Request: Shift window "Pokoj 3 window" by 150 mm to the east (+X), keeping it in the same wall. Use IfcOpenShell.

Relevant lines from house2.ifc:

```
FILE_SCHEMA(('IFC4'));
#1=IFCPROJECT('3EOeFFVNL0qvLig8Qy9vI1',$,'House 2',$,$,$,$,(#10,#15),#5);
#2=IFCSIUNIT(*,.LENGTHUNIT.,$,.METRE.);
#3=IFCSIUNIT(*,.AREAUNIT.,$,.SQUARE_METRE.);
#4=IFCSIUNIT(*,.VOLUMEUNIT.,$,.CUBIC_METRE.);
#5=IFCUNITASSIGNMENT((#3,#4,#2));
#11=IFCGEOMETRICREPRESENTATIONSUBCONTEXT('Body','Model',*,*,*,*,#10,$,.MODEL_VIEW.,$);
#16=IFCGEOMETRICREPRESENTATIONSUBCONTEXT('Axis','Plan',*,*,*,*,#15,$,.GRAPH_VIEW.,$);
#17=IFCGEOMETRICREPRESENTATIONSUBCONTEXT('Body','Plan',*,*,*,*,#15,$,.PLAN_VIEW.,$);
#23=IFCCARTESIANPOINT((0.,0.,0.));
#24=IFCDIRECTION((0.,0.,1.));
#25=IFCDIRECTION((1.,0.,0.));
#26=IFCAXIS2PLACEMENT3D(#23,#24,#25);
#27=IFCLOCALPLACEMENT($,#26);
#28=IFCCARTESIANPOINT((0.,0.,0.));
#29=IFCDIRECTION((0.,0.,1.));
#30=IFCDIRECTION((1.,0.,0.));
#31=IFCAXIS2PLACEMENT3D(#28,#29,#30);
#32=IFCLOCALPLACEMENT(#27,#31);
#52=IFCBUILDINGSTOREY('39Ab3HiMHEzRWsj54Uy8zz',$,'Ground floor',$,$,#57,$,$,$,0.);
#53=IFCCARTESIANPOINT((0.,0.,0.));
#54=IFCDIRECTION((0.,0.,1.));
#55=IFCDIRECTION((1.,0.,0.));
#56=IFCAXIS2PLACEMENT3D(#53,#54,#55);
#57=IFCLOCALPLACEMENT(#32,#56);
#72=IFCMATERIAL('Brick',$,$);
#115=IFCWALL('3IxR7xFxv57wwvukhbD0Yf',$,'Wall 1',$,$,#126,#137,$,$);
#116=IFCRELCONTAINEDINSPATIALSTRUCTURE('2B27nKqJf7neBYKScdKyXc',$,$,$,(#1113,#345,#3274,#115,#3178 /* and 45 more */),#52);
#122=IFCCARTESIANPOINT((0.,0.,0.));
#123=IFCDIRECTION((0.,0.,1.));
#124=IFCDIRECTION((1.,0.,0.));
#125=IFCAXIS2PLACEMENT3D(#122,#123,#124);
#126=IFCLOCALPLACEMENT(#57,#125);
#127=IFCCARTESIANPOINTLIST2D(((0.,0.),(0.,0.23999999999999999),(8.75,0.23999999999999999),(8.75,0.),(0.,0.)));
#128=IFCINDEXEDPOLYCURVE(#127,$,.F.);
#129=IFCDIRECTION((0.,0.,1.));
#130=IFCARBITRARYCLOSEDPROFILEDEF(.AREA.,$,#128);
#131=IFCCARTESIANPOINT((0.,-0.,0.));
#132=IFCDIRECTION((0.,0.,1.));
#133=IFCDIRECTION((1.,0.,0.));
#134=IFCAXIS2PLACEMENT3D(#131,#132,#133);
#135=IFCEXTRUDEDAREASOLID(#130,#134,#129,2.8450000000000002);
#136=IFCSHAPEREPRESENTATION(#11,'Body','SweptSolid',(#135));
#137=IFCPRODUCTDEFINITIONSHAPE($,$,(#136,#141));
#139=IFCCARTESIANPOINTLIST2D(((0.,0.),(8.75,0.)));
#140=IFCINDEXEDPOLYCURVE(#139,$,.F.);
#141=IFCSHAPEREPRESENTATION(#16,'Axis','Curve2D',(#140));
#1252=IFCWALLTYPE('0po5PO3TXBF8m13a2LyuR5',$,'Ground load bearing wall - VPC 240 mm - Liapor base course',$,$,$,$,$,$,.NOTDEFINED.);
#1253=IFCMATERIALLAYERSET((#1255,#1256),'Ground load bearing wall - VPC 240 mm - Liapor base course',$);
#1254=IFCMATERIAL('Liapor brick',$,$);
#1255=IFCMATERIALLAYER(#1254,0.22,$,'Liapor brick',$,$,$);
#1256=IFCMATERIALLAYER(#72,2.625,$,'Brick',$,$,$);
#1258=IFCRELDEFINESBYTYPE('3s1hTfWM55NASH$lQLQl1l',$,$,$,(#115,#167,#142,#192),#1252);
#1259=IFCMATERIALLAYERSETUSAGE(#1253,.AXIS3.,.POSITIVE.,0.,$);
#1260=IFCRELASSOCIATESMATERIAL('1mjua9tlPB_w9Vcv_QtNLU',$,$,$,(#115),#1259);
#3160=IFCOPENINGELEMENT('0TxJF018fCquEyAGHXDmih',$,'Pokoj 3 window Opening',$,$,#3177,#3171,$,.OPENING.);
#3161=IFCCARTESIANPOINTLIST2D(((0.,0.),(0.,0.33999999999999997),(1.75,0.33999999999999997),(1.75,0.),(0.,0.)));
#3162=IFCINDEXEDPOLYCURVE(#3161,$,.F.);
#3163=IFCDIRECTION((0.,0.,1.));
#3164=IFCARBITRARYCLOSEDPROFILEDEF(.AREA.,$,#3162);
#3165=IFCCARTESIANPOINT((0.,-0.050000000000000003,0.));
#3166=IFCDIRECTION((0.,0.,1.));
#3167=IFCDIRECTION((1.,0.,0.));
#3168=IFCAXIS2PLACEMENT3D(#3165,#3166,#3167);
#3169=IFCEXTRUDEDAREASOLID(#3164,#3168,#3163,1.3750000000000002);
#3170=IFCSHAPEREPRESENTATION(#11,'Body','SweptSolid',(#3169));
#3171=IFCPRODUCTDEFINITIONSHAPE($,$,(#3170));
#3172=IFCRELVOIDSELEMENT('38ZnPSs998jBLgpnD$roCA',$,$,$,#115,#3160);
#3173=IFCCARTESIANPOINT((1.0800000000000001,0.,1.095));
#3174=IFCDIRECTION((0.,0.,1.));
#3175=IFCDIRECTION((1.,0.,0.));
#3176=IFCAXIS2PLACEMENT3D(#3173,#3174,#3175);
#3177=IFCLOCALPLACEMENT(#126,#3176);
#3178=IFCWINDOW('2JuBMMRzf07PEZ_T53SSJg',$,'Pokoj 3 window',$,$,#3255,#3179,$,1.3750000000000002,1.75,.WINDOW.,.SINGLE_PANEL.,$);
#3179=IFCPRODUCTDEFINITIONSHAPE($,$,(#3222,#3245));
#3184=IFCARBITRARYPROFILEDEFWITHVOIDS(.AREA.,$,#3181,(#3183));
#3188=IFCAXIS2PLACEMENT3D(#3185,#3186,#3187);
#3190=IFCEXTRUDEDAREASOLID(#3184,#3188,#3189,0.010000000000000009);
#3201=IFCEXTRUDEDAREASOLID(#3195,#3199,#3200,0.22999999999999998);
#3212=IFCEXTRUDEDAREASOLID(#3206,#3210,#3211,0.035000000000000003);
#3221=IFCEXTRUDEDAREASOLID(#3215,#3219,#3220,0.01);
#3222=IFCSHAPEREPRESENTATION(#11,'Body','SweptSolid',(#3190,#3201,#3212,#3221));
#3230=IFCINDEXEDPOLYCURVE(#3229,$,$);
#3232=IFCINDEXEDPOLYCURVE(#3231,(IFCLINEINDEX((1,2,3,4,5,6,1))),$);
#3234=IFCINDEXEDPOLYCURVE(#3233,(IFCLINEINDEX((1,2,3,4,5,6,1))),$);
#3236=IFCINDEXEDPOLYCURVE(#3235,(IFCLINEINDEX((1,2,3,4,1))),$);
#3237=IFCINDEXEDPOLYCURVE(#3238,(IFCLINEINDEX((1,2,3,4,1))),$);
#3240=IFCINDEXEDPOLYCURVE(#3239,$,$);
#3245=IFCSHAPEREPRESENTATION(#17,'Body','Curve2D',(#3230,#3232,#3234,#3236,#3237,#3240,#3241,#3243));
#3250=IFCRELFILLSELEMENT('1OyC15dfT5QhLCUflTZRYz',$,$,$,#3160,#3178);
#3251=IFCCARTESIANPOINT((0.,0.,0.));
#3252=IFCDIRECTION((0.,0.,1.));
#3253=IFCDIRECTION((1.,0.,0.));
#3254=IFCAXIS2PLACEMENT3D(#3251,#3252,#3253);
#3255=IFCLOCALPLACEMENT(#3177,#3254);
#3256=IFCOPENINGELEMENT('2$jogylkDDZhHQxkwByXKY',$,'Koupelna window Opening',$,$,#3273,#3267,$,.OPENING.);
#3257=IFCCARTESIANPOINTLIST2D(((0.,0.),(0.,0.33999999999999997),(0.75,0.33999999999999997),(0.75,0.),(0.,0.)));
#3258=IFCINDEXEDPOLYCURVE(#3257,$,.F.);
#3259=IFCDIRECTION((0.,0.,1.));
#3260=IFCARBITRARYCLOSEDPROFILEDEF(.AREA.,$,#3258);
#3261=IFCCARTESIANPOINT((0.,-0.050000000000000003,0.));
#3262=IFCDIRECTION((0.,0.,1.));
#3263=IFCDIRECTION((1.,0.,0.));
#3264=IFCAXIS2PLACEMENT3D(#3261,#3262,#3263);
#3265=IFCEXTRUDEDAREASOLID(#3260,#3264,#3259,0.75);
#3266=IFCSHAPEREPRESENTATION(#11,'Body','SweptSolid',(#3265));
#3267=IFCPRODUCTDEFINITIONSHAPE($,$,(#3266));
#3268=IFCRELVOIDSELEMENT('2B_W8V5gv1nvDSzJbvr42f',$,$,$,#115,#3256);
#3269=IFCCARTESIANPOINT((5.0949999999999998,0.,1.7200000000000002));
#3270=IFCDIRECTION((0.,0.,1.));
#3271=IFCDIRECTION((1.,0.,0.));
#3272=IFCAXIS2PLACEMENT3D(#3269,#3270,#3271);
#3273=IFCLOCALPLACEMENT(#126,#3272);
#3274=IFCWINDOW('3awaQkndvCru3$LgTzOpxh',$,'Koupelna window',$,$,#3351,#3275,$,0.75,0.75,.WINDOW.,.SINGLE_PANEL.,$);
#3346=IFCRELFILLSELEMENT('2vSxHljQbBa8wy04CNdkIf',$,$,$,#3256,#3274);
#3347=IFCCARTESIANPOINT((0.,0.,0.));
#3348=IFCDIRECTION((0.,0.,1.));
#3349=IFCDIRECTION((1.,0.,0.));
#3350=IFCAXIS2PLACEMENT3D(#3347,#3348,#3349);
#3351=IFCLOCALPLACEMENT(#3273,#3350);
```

```python
import ifcopenshell
import ifcopenshell.api.geometry
import ifcopenshell.util.placement

model = ifcopenshell.open("house2.ifc")

window = model.by_guid("2JuBMMRzf07PEZ_T53SSJg")
opening = window.FillsVoids[0].RelatingOpeningElement
wall = opening.VoidsElements[0].RelatingBuildingElement

wall_matrix = ifcopenshell.util.placement.get_local_placement(wall.ObjectPlacement)
shift = wall_matrix[:3, 0] * 0.15
before = ifcopenshell.util.placement.get_local_placement(window.ObjectPlacement)[:3, 3].copy()

# The window is placed relative to its opening, so it follows when the opening moves.
matrix = ifcopenshell.util.placement.get_local_placement(opening.ObjectPlacement)
matrix[:3, 3] += shift
ifcopenshell.api.geometry.edit_object_placement(
    model, product=opening, matrix=matrix, is_si=False, should_transform_children=True
)

after = ifcopenshell.util.placement.get_local_placement(window.ObjectPlacement)[:3, 3]
print("window moved by", (after - before).round(3) + 0.0)

model.write("house2_updated.ifc")
```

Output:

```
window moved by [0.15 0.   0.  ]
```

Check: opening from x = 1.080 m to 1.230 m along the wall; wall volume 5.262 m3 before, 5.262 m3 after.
